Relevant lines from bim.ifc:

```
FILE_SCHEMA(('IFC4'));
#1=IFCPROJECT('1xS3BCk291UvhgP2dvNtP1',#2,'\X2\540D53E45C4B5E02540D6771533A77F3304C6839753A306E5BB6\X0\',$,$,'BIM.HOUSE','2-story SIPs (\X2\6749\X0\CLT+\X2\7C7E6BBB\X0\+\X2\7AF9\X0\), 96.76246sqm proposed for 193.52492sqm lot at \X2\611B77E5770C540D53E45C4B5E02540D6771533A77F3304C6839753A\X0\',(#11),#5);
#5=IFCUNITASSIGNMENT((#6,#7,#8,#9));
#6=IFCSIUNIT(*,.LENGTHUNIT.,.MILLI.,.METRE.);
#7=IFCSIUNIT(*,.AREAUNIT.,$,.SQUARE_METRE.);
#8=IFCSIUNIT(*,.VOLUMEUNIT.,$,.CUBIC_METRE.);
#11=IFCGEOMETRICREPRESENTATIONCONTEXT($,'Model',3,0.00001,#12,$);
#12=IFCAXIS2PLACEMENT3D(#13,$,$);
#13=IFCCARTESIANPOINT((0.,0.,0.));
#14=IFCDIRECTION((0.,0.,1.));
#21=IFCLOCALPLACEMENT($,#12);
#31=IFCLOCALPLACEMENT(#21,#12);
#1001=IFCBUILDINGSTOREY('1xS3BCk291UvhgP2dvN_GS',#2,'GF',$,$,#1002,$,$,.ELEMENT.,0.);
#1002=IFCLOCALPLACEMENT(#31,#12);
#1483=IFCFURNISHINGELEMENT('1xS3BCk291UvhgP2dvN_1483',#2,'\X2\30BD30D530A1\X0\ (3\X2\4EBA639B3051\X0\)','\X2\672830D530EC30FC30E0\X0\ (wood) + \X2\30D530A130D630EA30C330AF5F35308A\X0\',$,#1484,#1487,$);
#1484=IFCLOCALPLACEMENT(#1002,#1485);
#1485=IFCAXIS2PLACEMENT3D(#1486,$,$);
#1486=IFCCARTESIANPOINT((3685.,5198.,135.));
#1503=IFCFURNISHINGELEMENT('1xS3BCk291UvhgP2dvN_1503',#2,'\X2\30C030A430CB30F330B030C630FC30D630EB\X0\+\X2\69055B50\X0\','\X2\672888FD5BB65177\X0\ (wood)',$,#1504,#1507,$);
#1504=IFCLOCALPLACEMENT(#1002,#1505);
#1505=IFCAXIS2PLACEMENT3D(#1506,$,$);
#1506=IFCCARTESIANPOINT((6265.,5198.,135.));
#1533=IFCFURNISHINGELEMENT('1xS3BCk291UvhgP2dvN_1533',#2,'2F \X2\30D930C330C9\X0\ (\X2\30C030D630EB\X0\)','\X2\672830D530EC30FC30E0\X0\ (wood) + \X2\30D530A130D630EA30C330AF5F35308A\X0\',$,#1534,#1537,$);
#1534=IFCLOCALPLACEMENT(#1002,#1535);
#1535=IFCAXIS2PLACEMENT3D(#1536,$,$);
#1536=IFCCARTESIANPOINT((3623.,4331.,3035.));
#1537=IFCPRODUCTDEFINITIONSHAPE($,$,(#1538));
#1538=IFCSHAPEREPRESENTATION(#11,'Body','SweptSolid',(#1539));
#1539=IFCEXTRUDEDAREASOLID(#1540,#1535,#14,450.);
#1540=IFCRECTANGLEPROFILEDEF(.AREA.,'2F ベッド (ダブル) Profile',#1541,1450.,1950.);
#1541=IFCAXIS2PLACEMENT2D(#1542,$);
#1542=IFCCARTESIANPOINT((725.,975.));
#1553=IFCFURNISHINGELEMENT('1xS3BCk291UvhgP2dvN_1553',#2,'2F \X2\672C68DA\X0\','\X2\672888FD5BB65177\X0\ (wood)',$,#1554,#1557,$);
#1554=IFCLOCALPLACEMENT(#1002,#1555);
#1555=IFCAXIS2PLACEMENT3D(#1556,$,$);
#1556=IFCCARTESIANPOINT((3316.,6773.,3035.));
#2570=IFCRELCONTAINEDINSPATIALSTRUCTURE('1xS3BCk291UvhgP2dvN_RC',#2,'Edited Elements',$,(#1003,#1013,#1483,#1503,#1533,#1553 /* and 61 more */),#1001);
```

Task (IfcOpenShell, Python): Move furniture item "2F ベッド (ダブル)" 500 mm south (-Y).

```python
import ifcopenshell
import ifcopenshell.api.geometry
import ifcopenshell.util.placement
import ifcopenshell.util.unit

model = ifcopenshell.open("bim.ifc")
unit_scale = ifcopenshell.util.unit.calculate_unit_scale(model)

item = model.by_id(1533)
matrix = ifcopenshell.util.placement.get_local_placement(item.ObjectPlacement)
matrix[1, 3] -= 0.5 / unit_scale
ifcopenshell.api.geometry.edit_object_placement(model, product=item, matrix=matrix, is_si=False)

print(ifcopenshell.util.placement.get_local_placement(item.ObjectPlacement).round(3) + 0.0)

model.write("bim_v2.ifc")
```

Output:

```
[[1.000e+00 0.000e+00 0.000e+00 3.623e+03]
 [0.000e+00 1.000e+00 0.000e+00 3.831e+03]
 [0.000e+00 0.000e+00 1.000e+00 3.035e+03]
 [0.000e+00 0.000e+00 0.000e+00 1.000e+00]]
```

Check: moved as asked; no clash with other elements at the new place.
